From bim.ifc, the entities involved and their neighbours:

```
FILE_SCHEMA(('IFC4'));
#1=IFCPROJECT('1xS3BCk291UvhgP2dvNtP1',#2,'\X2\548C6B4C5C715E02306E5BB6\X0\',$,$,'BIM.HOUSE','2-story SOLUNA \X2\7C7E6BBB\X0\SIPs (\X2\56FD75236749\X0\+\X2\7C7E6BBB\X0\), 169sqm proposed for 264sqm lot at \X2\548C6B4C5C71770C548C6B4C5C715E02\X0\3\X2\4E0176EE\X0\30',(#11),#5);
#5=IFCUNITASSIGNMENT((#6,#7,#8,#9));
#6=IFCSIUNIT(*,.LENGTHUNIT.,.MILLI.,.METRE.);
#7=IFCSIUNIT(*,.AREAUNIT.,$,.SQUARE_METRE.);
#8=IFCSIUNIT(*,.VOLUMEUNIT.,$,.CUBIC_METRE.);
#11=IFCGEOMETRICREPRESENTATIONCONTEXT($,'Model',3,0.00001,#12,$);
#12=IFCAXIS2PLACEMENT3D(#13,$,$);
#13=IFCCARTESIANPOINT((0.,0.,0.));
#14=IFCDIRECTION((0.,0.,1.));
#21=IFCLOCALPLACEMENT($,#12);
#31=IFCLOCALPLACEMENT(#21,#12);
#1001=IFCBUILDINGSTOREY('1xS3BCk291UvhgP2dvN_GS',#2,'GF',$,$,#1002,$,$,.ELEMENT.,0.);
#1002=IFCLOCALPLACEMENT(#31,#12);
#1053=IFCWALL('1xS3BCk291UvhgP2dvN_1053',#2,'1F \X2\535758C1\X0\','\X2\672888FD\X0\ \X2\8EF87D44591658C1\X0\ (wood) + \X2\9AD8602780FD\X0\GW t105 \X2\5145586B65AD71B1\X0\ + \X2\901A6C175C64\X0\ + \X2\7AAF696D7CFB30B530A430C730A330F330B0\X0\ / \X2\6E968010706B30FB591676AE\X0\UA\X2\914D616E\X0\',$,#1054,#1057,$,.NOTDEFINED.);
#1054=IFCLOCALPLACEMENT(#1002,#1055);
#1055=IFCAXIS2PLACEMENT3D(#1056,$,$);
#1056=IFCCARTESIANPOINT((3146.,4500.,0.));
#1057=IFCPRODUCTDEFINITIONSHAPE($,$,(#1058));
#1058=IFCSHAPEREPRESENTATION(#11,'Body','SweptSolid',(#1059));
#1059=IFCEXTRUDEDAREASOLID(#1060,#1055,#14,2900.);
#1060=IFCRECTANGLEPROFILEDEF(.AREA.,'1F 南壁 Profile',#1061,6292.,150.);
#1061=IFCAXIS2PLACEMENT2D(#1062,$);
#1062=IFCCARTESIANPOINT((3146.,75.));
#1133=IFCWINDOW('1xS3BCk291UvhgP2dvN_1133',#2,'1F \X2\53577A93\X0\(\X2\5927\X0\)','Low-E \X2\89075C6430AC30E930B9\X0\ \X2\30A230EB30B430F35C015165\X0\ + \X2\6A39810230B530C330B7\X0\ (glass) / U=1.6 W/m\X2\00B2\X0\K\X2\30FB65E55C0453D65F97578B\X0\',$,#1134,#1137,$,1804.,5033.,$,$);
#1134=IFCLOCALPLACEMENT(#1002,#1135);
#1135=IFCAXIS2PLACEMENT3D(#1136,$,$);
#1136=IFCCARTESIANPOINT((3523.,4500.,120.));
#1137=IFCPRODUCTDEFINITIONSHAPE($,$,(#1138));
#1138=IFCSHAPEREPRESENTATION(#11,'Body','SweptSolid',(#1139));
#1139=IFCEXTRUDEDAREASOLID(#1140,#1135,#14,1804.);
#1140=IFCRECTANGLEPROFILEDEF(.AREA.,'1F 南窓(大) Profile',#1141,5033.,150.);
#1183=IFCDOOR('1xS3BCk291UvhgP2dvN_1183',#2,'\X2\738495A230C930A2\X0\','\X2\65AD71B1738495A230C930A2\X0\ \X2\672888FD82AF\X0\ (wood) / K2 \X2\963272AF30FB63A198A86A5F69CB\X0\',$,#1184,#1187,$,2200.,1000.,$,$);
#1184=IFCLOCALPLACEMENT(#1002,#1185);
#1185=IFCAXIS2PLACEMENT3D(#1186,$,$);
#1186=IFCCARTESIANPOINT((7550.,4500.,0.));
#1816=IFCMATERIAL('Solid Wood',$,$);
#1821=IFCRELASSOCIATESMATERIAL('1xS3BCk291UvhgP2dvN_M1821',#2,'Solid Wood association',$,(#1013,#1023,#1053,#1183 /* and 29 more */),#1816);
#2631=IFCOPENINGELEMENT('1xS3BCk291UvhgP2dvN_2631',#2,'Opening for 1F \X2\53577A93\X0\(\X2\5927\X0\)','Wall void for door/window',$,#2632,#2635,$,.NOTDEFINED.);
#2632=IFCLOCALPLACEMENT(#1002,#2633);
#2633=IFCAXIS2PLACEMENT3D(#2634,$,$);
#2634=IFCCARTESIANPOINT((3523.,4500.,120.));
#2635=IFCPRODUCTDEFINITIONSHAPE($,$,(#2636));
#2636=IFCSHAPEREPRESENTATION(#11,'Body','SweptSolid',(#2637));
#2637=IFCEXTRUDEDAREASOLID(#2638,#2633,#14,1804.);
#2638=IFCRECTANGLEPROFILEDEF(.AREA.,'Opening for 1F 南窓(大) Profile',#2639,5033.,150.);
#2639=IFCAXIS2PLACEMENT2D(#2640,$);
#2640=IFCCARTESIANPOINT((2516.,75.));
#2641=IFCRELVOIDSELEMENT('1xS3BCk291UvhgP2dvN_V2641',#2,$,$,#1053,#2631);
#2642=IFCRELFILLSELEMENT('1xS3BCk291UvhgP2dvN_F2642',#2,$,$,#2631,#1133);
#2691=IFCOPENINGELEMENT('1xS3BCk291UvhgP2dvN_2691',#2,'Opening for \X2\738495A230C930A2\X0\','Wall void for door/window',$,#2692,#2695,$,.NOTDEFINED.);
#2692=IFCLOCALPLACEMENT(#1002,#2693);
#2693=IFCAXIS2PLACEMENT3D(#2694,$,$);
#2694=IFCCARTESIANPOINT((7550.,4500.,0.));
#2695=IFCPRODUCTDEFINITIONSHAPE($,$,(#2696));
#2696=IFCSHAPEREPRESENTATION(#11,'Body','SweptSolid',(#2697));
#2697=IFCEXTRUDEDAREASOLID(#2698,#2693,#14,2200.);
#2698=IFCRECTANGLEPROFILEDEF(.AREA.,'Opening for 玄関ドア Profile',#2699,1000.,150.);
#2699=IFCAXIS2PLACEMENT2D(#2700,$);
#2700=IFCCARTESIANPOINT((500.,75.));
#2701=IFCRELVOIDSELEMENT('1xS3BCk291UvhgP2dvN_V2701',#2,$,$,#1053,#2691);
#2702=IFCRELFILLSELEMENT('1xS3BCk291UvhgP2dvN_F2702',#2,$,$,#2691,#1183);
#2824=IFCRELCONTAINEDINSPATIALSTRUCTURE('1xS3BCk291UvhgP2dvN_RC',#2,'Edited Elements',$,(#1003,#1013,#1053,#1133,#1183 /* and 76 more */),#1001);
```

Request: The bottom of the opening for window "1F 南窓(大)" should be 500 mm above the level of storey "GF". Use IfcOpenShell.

```python
import numpy as np
import ifcopenshell
import ifcopenshell.api.geometry
import ifcopenshell.geom
import ifcopenshell.util.element
import ifcopenshell.util.placement
import ifcopenshell.util.shape
import ifcopenshell.util.unit

model = ifcopenshell.open("bim.ifc")
unit_scale = ifcopenshell.util.unit.calculate_unit_scale(model)

window = model.by_id(1133)
opening = window.FillsVoids[0].RelatingOpeningElement
storey = ifcopenshell.util.element.get_container(window, ifc_class="IfcBuildingStorey")
level = ifcopenshell.util.placement.get_local_placement(storey.ObjectPlacement)[2, 3]

# The opening's origin need not be at the sill, so measure its lowest point.
shape = ifcopenshell.geom.create_shape(ifcopenshell.geom.settings(), opening)
bottom = ifcopenshell.util.shape.get_shape_bottom_elevation(shape, shape.geometry) / unit_scale
dz = level + 0.5 / unit_scale - bottom

shift = np.array([0.0, 0.0, dz])
# The window is not placed relative to its opening, so move both.
for product in (opening, window):
    matrix = ifcopenshell.util.placement.get_local_placement(product.ObjectPlacement)
    matrix[:3, 3] += shift
    ifcopenshell.api.geometry.edit_object_placement(model, product=product, matrix=matrix, is_si=False)

print(f"moved by {dz * unit_scale:+.3f} m")

model.write("bim_updated.ifc")
```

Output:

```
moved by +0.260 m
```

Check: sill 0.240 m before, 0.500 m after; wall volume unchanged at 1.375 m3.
